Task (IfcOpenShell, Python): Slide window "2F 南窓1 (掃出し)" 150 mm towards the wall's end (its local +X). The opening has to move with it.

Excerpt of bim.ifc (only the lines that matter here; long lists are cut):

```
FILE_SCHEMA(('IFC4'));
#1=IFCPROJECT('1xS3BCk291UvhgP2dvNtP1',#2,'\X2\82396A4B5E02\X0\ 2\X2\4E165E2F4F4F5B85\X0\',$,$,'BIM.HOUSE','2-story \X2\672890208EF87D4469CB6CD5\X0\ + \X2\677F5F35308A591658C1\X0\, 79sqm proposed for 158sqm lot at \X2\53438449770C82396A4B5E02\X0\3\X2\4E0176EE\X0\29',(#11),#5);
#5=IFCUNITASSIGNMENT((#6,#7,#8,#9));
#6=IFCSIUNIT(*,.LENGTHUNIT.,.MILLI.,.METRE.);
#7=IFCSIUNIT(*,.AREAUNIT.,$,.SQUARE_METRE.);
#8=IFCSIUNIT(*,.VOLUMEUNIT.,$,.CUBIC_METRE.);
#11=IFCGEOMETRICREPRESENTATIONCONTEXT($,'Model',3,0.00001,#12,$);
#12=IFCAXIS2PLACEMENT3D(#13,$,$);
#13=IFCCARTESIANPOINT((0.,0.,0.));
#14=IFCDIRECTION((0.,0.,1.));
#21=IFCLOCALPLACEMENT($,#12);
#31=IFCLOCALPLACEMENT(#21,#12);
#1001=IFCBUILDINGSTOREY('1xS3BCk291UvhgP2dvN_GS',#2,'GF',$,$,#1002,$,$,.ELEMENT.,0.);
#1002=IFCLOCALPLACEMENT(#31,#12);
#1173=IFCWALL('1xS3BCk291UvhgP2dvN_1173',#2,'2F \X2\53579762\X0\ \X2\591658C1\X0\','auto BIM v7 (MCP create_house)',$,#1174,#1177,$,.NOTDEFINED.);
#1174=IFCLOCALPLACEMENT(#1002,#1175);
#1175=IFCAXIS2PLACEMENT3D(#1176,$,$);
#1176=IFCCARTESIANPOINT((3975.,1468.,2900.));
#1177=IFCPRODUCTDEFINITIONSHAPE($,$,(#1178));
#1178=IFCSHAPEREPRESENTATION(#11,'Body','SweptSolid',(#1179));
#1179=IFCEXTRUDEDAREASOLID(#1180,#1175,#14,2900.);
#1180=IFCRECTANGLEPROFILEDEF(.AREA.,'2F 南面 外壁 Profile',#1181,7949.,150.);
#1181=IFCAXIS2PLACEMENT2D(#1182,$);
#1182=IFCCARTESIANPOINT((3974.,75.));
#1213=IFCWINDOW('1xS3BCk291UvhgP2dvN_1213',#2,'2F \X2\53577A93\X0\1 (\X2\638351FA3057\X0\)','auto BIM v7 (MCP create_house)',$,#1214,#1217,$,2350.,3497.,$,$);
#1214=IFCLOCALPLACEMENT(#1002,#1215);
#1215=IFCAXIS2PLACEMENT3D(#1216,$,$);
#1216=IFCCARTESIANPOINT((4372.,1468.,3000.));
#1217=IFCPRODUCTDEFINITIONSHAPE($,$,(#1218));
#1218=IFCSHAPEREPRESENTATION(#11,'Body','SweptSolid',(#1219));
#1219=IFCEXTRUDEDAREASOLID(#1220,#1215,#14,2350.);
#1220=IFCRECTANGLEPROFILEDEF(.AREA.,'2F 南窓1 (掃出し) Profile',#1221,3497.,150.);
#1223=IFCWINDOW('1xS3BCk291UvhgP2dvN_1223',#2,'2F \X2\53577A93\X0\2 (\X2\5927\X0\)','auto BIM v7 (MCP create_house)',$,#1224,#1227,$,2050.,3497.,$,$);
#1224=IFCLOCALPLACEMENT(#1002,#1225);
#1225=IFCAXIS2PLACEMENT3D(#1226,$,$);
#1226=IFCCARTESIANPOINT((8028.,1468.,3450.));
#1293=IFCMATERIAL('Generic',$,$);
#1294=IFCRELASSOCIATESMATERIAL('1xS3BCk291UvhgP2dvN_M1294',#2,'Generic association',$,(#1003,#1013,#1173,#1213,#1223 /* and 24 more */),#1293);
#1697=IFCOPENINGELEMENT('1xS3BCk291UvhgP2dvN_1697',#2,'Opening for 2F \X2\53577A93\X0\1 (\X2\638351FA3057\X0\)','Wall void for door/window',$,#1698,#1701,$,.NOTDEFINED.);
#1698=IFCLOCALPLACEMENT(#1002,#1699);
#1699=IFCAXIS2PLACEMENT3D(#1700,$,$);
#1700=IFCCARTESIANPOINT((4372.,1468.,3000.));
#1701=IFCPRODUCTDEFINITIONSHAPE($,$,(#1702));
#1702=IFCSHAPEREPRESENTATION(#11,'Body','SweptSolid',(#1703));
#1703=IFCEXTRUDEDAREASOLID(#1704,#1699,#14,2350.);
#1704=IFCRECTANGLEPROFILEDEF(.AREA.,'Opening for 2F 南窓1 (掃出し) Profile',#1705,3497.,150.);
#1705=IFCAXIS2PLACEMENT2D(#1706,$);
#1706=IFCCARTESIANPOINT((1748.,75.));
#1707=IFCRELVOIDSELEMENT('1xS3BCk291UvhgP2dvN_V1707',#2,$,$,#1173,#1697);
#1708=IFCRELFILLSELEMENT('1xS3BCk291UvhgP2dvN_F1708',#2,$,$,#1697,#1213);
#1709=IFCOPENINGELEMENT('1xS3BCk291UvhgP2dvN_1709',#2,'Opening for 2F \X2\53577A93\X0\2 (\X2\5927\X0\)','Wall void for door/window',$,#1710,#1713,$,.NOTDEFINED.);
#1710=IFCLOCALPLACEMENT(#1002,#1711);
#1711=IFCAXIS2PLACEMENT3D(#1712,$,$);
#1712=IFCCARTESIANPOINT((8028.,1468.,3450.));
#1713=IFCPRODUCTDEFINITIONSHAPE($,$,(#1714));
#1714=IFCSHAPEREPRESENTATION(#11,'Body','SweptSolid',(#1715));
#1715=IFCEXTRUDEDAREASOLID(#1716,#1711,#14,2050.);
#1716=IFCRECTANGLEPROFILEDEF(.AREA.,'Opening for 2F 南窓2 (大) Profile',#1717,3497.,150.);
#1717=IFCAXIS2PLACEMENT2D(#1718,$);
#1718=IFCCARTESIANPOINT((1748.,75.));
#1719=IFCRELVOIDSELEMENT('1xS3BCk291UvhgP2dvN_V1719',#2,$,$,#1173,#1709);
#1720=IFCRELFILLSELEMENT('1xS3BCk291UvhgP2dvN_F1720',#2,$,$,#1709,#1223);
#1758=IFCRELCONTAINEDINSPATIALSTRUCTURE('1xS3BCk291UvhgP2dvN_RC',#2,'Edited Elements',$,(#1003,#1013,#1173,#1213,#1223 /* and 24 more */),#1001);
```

```python
import ifcopenshell
import ifcopenshell.api.geometry
import ifcopenshell.util.placement
import ifcopenshell.util.unit

model = ifcopenshell.open("bim.ifc")
unit_scale = ifcopenshell.util.unit.calculate_unit_scale(model)

window = model.by_guid("1xS3BCk291UvhgP2dvN_1213")
opening = window.FillsVoids[0].RelatingOpeningElement
wall = opening.VoidsElements[0].RelatingBuildingElement

wall_matrix = ifcopenshell.util.placement.get_local_placement(wall.ObjectPlacement)
shift = wall_matrix[:3, 0] * 0.15 / unit_scale
before = ifcopenshell.util.placement.get_local_placement(window.ObjectPlacement)[:3, 3].copy()

# The window is not placed relative to its opening, so move both.
for product in (opening, window):
    matrix = ifcopenshell.util.placement.get_local_placement(product.ObjectPlacement)
    matrix[:3, 3] += shift
    ifcopenshell.api.geometry.edit_object_placement(model, product=product, matrix=matrix, is_si=False)

after = ifcopenshell.util.placement.get_local_placement(window.ObjectPlacement)[:3, 3]
print("window moved by", (after - before).round(3) + 0.0)

model.write("bim_v2.ifc")
```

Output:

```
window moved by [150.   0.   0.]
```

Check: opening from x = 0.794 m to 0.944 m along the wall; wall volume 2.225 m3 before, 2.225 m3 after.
